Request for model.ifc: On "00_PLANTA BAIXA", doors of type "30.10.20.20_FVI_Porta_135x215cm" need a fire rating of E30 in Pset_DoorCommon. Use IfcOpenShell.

First a look at what the model holds.

```python
import ifcopenshell
import ifcopenshell.util.element

model = ifcopenshell.open("model.ifc")
print(model.schema)
storey = next(s for s in model.by_type("IfcBuildingStorey") if s.Name == "00_PLANTA BAIXA")
doors = [e for e in ifcopenshell.util.element.get_decomposition(storey) if e.is_a("IfcDoor")]
seen = {}
for e in doors:
    element_type = ifcopenshell.util.element.get_type(e)
    key = (element_type.Name if element_type != e and element_type else None, ifcopenshell.util.element.get_pset(e, "Pset_DoorCommon", "FireRating"))
    seen[key] = seen.get(key, 0) + 1
for (name, value), count in sorted(seen.items(), key=str):
    print(count, "x", name, "|", value)
```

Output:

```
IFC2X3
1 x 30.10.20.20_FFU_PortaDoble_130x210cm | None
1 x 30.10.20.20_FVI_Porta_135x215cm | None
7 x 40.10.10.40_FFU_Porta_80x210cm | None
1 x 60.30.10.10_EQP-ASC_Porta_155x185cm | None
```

```python
import ifcopenshell
import ifcopenshell.api.pset
import ifcopenshell.util.element

model = ifcopenshell.open("model.ifc")

storey = next(s for s in model.by_type("IfcBuildingStorey") if s.Name == "00_PLANTA BAIXA")
doors = [e for e in ifcopenshell.util.element.get_decomposition(storey) if e.is_a("IfcDoor")]

count = 0
for e in doors:
    element_type = ifcopenshell.util.element.get_type(e)
    if element_type in (None, e) or element_type.Name != "30.10.20.20_FVI_Porta_135x215cm":
        continue
    # add_pset returns the element's existing set when there is one.
    pset = ifcopenshell.api.pset.add_pset(model, product=e, name="Pset_DoorCommon")
    ifcopenshell.api.pset.edit_pset(model, pset=pset, properties={"FireRating": "E30"})
    count += 1

print(count, "doors updated")

model.write("model-out.ifc")
```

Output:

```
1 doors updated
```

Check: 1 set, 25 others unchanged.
